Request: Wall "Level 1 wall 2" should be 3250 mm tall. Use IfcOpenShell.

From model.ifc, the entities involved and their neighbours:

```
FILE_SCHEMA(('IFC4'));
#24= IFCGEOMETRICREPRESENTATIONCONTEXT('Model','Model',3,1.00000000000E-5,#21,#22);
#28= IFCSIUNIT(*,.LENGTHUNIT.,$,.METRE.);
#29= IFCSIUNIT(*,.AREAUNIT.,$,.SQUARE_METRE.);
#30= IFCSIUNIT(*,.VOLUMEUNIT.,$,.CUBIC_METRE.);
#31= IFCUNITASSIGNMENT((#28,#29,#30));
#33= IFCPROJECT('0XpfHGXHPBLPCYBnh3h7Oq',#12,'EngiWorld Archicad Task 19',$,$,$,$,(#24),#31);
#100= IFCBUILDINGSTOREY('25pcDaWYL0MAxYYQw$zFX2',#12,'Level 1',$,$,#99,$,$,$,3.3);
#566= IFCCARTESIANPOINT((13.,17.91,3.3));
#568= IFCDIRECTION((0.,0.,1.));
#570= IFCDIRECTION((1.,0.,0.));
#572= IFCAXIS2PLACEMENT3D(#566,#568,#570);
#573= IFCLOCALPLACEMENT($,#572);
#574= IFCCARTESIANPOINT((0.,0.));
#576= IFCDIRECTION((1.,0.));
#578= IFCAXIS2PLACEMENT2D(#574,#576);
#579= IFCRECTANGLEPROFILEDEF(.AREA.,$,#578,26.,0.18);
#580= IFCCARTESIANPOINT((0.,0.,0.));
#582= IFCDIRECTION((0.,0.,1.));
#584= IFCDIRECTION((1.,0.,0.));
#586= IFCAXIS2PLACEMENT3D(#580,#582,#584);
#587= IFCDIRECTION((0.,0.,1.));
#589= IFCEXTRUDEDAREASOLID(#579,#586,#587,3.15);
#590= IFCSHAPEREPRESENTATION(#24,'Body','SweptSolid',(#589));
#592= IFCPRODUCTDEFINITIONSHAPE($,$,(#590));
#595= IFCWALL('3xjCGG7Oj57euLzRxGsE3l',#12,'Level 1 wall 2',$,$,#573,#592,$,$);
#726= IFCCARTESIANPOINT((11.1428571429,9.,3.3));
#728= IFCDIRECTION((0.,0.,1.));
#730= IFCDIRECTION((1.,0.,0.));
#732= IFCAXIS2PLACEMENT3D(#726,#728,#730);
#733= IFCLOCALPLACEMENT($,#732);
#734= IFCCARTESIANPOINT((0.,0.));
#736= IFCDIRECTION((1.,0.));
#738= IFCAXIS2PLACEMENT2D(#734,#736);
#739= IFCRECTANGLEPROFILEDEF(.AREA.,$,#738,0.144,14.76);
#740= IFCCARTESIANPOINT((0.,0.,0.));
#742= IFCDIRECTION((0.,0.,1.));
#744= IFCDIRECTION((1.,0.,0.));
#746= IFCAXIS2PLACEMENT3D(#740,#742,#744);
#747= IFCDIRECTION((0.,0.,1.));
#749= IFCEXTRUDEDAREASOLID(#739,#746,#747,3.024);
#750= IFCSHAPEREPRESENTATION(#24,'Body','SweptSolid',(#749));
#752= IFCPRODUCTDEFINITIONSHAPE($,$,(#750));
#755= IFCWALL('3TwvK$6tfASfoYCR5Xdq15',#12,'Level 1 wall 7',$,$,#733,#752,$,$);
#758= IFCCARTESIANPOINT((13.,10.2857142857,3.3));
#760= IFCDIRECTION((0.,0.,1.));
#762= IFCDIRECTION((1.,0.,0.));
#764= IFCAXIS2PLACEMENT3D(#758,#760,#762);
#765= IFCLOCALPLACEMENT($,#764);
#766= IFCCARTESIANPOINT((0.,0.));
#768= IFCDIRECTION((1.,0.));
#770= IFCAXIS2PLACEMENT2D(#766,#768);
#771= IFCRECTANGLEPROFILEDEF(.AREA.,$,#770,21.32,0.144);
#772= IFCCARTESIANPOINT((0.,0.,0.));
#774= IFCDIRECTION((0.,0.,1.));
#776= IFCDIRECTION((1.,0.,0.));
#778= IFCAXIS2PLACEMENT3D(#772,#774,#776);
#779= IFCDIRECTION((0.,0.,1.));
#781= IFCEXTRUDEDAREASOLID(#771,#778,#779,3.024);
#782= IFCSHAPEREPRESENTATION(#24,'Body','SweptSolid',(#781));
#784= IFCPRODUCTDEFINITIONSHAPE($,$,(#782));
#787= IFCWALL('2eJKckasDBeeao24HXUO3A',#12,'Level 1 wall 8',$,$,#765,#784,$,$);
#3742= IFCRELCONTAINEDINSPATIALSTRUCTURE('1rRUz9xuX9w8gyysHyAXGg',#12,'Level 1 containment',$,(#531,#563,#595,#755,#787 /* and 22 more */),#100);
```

```python
import ifcopenshell
import ifcopenshell.geom
import ifcopenshell.util.shape
import ifcopenshell.util.unit

model = ifcopenshell.open("model.ifc")
unit_scale = ifcopenshell.util.unit.calculate_unit_scale(model)
settings = ifcopenshell.geom.settings()


def volume(element):
    """Net volume in cubic metres, openings subtracted."""
    shape = ifcopenshell.geom.create_shape(settings, element)
    return ifcopenshell.util.shape.get_volume(shape.geometry)


wall = model.by_id(595)
before = volume(wall)

body = next(r for r in wall.Representation.Representations if r.RepresentationIdentifier == "Body")
solid = body.Items[0]
old_height = solid.Depth
solid.Depth = 3.25 / unit_scale
after = volume(wall)

print(f"height {old_height:g} -> {solid.Depth:g}, volume {before:.3f} -> {after:.3f} m3")

model.write("model_v2.ifc")
```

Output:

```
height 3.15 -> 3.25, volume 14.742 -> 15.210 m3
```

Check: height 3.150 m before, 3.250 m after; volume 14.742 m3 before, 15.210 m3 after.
